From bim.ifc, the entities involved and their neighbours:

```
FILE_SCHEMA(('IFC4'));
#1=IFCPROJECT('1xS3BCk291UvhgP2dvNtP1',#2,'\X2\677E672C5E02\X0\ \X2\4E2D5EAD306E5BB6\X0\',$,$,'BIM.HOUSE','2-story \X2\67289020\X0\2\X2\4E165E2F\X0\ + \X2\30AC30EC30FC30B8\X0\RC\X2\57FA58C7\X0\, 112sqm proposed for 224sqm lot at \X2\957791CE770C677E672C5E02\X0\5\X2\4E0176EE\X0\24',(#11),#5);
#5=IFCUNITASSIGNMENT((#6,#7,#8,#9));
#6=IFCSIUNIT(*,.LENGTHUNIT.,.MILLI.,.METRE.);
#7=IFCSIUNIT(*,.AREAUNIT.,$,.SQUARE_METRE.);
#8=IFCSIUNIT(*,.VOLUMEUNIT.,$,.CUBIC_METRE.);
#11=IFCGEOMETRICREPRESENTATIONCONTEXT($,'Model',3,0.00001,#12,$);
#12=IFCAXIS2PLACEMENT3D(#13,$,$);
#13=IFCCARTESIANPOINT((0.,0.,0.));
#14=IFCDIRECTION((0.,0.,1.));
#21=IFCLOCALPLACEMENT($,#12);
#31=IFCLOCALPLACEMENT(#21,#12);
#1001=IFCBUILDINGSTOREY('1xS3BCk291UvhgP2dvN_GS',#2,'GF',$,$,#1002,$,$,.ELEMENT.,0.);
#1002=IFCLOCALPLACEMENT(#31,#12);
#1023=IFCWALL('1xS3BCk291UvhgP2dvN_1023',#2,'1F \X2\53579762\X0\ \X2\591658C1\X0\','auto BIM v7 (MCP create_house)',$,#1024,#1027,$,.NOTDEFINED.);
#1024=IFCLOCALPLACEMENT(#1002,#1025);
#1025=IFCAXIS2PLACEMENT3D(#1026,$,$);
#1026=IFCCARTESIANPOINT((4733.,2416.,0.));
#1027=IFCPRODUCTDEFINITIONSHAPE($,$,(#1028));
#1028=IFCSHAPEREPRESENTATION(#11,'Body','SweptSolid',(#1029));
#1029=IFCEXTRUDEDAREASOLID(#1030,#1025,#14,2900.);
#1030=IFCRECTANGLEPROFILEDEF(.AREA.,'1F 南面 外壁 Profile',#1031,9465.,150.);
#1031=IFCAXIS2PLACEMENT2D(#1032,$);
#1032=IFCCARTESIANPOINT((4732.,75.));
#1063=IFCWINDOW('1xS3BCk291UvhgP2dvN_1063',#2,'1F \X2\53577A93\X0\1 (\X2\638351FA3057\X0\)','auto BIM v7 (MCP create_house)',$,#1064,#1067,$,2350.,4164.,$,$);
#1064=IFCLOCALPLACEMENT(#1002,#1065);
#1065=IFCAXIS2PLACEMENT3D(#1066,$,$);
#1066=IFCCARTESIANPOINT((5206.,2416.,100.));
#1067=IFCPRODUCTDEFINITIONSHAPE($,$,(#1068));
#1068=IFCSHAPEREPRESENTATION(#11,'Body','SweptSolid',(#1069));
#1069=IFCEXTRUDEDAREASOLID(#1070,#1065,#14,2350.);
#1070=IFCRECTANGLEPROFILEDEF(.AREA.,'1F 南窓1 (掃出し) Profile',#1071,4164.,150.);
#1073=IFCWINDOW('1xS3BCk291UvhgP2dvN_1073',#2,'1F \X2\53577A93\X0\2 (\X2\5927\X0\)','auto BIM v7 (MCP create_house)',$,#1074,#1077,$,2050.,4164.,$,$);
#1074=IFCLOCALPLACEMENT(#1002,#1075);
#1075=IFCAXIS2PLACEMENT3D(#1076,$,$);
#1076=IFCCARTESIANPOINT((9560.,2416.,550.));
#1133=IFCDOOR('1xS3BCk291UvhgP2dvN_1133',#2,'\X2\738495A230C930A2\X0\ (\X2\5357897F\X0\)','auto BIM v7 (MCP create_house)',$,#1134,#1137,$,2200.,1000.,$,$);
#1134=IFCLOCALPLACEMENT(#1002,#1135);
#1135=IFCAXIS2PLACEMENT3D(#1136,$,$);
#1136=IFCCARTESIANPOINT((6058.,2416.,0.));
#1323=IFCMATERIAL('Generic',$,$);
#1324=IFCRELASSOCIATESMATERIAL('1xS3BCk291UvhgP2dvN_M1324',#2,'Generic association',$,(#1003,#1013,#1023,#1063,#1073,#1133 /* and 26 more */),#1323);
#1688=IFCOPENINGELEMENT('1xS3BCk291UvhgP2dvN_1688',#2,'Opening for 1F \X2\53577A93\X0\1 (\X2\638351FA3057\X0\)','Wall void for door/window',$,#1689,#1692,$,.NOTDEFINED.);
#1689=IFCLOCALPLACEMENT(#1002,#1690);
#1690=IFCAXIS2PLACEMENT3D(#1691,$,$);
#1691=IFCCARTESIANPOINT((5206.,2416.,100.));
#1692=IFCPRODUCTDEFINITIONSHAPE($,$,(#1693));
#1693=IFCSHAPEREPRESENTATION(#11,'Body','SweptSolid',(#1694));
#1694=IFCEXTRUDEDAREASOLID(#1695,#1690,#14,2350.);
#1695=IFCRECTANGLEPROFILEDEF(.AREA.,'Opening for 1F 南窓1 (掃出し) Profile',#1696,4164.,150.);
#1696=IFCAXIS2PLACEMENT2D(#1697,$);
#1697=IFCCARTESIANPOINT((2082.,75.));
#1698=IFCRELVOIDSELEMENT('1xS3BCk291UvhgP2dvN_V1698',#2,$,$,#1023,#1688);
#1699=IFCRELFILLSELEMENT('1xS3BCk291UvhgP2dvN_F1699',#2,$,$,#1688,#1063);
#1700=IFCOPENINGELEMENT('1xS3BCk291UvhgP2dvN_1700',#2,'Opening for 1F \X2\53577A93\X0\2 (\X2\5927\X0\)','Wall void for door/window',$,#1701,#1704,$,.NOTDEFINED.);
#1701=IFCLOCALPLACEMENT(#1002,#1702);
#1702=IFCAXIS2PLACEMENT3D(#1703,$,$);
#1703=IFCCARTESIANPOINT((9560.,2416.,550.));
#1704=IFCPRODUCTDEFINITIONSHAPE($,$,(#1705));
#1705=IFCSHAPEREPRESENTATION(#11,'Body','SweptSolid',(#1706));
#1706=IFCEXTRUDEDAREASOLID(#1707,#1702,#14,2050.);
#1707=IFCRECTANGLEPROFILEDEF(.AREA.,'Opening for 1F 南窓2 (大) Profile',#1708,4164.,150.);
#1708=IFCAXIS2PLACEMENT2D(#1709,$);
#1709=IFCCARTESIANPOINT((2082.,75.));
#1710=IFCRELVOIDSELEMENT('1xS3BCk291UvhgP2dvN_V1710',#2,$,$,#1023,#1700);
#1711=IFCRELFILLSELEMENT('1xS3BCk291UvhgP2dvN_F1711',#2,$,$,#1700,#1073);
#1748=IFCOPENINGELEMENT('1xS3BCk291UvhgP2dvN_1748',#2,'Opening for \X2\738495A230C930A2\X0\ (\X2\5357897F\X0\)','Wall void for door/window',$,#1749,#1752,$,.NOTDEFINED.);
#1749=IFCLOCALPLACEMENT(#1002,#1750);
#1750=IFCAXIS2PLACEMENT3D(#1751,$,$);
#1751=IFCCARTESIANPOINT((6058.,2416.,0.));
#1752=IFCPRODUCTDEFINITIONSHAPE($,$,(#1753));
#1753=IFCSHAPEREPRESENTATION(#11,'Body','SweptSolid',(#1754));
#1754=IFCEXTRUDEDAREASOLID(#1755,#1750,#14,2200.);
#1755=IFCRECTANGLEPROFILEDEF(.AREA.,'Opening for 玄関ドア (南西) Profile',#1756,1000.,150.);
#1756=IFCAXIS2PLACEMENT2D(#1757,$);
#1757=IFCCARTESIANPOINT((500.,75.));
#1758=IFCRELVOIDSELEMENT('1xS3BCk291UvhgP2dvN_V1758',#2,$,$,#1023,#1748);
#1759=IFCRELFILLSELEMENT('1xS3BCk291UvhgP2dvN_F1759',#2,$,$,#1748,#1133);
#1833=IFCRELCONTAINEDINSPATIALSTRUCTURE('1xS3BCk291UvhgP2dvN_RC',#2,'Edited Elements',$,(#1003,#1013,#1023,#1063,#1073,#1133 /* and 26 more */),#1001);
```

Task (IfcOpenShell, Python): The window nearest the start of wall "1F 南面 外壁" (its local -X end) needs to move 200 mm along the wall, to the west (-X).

```python
import ifcopenshell
import ifcopenshell.api.geometry
import ifcopenshell.util.placement
import ifcopenshell.util.unit

model = ifcopenshell.open("bim.ifc")
unit_scale = ifcopenshell.util.unit.calculate_unit_scale(model)

window = model.by_id(1063)
opening = window.FillsVoids[0].RelatingOpeningElement
wall = opening.VoidsElements[0].RelatingBuildingElement

wall_matrix = ifcopenshell.util.placement.get_local_placement(wall.ObjectPlacement)
shift = wall_matrix[:3, 0] * -0.2 / unit_scale
before = ifcopenshell.util.placement.get_local_placement(window.ObjectPlacement)[:3, 3].copy()

# The window is not placed relative to its opening, so move both.
for product in (opening, window):
    matrix = ifcopenshell.util.placement.get_local_placement(product.ObjectPlacement)
    matrix[:3, 3] += shift
    ifcopenshell.api.geometry.edit_object_placement(model, product=product, matrix=matrix, is_si=False)

after = ifcopenshell.util.placement.get_local_placement(window.ObjectPlacement)[:3, 3]
print("window moved by", (after - before).round(3) + 0.0)

model.write("bim_rev.ifc")
```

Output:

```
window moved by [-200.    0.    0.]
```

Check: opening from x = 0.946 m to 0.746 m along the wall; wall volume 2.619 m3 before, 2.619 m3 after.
